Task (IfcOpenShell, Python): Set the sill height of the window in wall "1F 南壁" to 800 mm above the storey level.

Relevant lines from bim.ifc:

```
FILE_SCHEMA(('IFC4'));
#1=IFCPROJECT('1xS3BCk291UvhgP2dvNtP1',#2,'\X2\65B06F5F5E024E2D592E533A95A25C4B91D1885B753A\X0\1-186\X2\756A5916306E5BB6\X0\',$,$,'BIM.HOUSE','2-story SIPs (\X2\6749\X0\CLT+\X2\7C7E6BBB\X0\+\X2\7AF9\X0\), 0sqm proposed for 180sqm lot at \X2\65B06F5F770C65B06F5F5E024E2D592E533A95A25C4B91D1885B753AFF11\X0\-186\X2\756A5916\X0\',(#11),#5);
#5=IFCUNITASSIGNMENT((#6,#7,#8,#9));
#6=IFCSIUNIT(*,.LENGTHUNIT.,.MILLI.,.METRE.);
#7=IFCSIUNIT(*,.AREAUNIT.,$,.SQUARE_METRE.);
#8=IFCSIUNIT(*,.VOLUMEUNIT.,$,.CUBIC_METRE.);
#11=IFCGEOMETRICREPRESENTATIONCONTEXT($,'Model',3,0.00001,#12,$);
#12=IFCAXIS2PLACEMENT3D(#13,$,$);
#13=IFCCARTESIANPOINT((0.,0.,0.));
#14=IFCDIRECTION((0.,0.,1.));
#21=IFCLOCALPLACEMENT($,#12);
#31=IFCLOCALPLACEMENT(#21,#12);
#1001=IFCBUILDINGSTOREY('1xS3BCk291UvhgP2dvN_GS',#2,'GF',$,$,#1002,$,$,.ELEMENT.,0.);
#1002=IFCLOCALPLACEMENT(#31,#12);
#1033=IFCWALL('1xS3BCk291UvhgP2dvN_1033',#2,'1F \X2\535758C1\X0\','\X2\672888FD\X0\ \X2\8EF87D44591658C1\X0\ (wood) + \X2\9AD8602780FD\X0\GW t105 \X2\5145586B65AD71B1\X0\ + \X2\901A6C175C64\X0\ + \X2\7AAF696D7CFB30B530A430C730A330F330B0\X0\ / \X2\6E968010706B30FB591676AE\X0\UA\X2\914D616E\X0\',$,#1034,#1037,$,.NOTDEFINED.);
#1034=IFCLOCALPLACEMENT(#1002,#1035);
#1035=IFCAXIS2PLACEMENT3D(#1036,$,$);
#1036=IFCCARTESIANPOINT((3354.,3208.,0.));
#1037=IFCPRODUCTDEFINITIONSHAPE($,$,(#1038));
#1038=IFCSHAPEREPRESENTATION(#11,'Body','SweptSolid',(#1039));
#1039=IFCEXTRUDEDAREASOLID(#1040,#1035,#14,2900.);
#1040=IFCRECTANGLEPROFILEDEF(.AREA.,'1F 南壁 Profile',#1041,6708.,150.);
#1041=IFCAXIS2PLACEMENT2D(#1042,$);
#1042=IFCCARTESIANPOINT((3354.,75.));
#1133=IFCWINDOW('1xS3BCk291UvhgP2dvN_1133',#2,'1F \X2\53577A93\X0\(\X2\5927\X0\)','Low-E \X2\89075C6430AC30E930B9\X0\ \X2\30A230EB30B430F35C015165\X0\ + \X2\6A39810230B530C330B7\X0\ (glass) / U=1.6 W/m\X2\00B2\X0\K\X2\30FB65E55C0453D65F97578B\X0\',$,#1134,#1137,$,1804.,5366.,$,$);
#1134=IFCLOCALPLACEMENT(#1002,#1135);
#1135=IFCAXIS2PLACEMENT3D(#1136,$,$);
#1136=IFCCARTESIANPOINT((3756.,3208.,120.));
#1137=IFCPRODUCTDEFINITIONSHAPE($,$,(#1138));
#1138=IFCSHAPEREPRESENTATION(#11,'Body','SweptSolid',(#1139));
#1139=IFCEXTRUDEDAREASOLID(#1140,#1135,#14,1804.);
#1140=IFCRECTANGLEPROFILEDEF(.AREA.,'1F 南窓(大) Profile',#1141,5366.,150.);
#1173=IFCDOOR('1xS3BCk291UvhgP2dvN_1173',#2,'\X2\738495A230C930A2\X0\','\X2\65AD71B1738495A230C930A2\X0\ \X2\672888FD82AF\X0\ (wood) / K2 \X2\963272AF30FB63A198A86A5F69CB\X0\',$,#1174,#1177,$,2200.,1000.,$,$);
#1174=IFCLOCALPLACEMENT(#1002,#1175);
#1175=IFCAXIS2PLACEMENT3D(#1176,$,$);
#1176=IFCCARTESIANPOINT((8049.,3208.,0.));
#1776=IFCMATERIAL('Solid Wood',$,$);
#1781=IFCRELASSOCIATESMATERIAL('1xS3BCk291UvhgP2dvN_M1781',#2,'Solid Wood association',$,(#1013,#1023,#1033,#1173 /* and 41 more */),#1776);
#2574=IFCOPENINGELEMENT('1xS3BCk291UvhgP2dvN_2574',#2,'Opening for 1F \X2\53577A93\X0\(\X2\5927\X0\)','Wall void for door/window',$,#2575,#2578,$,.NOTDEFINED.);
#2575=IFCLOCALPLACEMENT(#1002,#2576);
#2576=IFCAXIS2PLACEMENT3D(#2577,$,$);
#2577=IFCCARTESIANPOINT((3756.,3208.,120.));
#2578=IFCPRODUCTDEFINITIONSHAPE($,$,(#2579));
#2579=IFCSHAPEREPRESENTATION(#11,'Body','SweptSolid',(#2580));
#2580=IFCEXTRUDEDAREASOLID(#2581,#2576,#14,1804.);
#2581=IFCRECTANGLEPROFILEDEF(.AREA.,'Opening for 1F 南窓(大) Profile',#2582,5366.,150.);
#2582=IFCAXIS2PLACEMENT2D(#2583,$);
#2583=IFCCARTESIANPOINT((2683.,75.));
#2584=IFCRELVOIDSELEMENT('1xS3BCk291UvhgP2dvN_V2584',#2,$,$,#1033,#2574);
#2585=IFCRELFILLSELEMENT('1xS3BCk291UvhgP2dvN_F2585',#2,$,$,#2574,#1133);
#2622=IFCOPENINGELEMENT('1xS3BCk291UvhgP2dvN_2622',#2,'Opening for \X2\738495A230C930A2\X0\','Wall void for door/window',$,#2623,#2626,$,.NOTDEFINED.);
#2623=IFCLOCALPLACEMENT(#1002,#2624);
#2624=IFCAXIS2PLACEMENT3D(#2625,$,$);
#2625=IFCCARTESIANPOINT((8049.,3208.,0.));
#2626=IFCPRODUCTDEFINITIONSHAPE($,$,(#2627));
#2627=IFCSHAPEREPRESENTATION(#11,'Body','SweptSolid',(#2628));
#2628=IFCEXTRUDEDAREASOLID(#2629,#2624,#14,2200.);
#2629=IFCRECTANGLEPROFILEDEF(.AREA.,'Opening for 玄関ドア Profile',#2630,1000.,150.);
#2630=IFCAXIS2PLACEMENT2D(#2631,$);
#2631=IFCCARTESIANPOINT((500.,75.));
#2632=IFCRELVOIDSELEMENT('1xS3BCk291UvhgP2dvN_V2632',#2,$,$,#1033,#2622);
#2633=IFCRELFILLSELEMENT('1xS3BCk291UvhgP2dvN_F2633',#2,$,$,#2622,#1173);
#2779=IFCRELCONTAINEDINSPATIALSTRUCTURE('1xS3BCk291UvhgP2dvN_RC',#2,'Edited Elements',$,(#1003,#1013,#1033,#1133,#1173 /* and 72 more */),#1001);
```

```python
import numpy as np
import ifcopenshell
import ifcopenshell.api.geometry
import ifcopenshell.geom
import ifcopenshell.util.element
import ifcopenshell.util.placement
import ifcopenshell.util.shape
import ifcopenshell.util.unit

model = ifcopenshell.open("bim.ifc")
unit_scale = ifcopenshell.util.unit.calculate_unit_scale(model)

window = model.by_guid("1xS3BCk291UvhgP2dvN_1133")
opening = window.FillsVoids[0].RelatingOpeningElement
storey = ifcopenshell.util.element.get_container(window, ifc_class="IfcBuildingStorey")
level = ifcopenshell.util.placement.get_local_placement(storey.ObjectPlacement)[2, 3]

# The opening's origin need not be at the sill, so measure its lowest point.
shape = ifcopenshell.geom.create_shape(ifcopenshell.geom.settings(), opening)
bottom = ifcopenshell.util.shape.get_shape_bottom_elevation(shape, shape.geometry) / unit_scale
dz = level + 0.8 / unit_scale - bottom

shift = np.array([0.0, 0.0, dz])
# The window is not placed relative to its opening, so move both.
for product in (opening, window):
    matrix = ifcopenshell.util.placement.get_local_placement(product.ObjectPlacement)
    matrix[:3, 3] += shift
    ifcopenshell.api.geometry.edit_object_placement(model, product=product, matrix=matrix, is_si=False)

print(f"moved by {dz * unit_scale:+.3f} m")

model.write("bim_v2.ifc")
```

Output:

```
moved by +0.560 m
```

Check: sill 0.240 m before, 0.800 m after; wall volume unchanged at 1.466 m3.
